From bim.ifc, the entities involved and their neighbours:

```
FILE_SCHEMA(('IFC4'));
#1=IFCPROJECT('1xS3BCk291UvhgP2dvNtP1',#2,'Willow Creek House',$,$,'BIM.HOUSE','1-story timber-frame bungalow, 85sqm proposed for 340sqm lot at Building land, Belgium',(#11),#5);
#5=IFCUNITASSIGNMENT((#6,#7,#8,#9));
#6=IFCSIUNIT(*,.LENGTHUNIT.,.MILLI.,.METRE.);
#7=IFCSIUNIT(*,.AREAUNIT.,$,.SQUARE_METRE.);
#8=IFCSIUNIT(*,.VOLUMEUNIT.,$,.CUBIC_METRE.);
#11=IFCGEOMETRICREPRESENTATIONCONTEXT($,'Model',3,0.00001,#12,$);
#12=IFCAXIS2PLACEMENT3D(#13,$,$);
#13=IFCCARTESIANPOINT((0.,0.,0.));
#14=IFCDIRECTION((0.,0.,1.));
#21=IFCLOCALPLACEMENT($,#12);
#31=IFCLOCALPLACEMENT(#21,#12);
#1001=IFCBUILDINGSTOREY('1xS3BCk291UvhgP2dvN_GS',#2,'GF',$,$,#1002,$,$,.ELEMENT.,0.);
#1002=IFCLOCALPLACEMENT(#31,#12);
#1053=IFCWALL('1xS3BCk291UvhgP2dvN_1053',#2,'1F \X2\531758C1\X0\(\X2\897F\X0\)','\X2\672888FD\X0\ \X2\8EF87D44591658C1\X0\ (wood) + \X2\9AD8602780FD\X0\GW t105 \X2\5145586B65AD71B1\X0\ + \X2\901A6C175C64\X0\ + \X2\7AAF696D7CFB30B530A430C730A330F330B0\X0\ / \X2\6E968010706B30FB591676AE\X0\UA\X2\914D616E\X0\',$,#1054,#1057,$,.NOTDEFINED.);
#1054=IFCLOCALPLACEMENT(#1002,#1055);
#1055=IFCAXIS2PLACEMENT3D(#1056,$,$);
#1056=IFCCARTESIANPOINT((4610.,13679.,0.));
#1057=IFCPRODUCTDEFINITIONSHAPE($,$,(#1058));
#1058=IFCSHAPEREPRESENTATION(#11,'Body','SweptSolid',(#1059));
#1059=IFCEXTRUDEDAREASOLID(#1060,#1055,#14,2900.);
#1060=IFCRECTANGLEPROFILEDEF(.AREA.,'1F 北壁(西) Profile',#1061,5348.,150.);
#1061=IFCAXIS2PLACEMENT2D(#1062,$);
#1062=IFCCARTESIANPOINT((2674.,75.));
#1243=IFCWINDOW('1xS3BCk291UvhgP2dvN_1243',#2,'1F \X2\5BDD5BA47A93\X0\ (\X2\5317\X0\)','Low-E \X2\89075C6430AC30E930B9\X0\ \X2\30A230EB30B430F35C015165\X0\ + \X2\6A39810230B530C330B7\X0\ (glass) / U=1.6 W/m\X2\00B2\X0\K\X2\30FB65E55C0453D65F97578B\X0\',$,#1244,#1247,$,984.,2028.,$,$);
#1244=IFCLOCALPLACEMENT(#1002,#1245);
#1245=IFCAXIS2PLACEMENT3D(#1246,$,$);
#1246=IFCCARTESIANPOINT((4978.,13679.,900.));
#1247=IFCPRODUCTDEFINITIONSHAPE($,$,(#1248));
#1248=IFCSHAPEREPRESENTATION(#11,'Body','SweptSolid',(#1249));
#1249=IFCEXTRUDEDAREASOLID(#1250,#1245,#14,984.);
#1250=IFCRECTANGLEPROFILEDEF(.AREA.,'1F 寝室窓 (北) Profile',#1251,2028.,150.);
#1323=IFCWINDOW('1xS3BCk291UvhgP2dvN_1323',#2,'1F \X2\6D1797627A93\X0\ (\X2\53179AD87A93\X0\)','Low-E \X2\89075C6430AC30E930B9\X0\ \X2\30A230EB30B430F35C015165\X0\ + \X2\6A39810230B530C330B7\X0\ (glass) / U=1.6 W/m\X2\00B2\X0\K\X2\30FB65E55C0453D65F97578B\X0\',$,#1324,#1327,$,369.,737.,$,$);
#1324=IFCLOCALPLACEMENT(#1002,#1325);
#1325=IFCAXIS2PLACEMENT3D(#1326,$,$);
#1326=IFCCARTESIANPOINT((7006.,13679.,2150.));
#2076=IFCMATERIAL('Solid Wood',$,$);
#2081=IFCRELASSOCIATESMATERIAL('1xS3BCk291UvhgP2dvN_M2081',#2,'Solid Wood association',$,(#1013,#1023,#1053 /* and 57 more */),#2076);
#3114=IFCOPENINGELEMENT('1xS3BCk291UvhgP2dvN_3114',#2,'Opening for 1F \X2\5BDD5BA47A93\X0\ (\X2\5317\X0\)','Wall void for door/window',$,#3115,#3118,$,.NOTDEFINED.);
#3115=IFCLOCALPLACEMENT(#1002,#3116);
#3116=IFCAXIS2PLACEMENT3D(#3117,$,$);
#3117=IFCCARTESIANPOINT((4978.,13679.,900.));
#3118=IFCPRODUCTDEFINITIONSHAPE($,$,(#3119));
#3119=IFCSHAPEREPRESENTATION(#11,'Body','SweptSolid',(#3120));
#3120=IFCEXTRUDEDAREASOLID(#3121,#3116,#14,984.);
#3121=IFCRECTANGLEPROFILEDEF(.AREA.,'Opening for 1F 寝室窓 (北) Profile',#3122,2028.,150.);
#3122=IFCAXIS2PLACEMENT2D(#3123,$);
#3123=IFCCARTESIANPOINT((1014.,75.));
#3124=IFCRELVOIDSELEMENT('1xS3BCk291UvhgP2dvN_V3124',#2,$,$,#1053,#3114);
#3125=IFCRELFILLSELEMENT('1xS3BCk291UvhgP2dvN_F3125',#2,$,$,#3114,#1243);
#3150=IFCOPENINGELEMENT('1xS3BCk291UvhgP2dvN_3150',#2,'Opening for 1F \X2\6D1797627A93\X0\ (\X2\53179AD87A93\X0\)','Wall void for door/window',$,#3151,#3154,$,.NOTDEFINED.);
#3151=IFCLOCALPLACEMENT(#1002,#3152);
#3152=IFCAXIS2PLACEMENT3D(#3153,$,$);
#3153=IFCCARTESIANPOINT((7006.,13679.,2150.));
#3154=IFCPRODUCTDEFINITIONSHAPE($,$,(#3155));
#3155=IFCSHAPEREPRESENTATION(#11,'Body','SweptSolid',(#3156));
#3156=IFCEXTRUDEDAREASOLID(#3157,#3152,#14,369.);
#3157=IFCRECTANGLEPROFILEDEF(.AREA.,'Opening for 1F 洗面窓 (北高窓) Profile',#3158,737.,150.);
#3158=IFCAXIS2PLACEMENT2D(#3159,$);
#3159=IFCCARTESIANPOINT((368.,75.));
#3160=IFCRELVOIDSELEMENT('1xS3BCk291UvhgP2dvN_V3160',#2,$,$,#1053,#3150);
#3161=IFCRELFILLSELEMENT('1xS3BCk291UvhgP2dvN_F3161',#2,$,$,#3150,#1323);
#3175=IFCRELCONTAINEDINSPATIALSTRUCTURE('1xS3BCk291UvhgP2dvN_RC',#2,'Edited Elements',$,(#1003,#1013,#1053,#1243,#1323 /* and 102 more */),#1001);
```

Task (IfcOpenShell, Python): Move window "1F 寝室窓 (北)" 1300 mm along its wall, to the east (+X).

```python
import ifcopenshell
import ifcopenshell.api.geometry
import ifcopenshell.util.placement
import ifcopenshell.util.unit

model = ifcopenshell.open("bim.ifc")
unit_scale = ifcopenshell.util.unit.calculate_unit_scale(model)

window = model.by_guid("1xS3BCk291UvhgP2dvN_1243")
opening = window.FillsVoids[0].RelatingOpeningElement
wall = opening.VoidsElements[0].RelatingBuildingElement

wall_matrix = ifcopenshell.util.placement.get_local_placement(wall.ObjectPlacement)
shift = wall_matrix[:3, 0] * 1.3 / unit_scale
before = ifcopenshell.util.placement.get_local_placement(window.ObjectPlacement)[:3, 3].copy()

# The window is not placed relative to its opening, so move both.
for product in (opening, window):
    matrix = ifcopenshell.util.placement.get_local_placement(product.ObjectPlacement)
    matrix[:3, 3] += shift
    ifcopenshell.api.geometry.edit_object_placement(model, product=product, matrix=matrix, is_si=False)

after = ifcopenshell.util.placement.get_local_placement(window.ObjectPlacement)[:3, 3]
print("window moved by", (after - before).round(3) + 0.0)

model.write("bim_rev.ifc")
```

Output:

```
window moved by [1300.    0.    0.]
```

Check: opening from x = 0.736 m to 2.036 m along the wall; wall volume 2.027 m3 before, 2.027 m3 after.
